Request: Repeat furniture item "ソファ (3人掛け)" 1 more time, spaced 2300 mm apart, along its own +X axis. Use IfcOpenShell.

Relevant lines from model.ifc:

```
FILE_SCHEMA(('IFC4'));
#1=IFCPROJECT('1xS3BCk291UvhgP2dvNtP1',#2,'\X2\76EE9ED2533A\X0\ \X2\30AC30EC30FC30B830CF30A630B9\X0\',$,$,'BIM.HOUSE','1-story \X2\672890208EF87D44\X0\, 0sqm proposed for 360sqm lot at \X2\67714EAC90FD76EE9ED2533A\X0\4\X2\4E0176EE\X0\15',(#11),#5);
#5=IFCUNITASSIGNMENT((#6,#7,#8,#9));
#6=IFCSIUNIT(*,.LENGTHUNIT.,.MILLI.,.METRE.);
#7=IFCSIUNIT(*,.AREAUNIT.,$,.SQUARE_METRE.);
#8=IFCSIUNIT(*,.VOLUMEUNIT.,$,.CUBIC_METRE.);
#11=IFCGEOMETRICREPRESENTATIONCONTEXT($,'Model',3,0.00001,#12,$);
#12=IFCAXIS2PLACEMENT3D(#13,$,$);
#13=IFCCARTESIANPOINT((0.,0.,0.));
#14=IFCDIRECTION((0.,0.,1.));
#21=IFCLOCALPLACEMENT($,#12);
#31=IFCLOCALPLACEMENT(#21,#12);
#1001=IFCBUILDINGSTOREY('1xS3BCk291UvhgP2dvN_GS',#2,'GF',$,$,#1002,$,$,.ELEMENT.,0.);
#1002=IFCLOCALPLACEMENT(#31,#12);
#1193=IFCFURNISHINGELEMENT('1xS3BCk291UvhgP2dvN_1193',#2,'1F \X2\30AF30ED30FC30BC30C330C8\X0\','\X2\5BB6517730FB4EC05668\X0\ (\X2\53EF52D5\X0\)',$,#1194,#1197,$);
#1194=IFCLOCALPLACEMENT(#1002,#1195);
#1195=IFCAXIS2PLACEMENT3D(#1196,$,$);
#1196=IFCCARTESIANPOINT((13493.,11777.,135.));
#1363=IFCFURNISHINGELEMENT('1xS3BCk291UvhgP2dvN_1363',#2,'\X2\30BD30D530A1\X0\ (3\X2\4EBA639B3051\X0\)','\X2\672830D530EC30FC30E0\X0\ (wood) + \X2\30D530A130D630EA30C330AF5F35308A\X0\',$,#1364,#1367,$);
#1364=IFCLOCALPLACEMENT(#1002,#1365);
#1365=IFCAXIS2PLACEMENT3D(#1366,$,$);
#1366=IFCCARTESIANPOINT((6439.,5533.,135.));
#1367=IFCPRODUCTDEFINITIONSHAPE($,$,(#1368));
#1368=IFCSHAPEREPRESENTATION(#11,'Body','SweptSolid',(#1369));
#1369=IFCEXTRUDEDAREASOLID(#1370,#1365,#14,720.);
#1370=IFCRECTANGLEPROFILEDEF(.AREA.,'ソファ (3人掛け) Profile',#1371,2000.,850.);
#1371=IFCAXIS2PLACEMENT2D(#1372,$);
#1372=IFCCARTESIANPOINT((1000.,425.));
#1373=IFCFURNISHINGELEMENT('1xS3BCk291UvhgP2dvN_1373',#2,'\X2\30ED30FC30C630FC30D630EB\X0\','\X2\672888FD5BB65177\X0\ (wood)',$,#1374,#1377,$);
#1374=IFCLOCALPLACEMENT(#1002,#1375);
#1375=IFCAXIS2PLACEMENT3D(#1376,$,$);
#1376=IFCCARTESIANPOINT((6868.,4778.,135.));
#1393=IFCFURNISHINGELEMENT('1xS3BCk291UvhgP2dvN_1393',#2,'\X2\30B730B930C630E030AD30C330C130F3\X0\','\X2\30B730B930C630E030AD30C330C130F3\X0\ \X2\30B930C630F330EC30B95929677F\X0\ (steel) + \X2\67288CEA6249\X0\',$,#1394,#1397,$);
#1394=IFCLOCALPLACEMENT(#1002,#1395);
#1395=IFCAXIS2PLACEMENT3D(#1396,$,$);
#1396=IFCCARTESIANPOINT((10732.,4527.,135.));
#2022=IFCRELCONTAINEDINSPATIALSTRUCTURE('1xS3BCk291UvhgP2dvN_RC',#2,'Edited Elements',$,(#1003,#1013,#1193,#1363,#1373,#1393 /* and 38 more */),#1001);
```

```python
import ifcopenshell
import ifcopenshell.api.geometry
import ifcopenshell.api.root
import ifcopenshell.util.element
import ifcopenshell.util.placement

model = ifcopenshell.open("model.ifc")


def reuse_history(source, copy):
    """copy_class also copies each property set's owner history, people and application; keep the originals."""
    for rel in copy.IsDefinedBy:
        if rel.is_a("IfcRelDefinesByProperties") and (history := rel.RelatingPropertyDefinition.OwnerHistory):
            rel.RelatingPropertyDefinition.OwnerHistory = source.OwnerHistory
            ifcopenshell.util.element.remove_deep2(model, history)


source = model.by_guid("1xS3BCk291UvhgP2dvN_1363")
base = ifcopenshell.util.placement.get_local_placement(source.ObjectPlacement)
step = base[:3, 0] * 2300.0

for i in range(1, 2):
    copy = ifcopenshell.api.root.copy_class(model, product=source)
    copy.Representation = ifcopenshell.util.element.copy_deep(
        model, source.Representation, exclude=["IfcGeometricRepresentationContext", "IfcRepresentationMap"]
    )
    reuse_history(source, copy)
    matrix = base.copy()
    matrix[:3, 3] += i * step
    print("added at", matrix[:3, 3].round(3) + 0.0)
    ifcopenshell.api.geometry.edit_object_placement(model, product=copy, matrix=matrix, is_si=False)

model.write("model-out.ifc")
```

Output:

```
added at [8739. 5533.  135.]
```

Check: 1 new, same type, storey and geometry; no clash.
